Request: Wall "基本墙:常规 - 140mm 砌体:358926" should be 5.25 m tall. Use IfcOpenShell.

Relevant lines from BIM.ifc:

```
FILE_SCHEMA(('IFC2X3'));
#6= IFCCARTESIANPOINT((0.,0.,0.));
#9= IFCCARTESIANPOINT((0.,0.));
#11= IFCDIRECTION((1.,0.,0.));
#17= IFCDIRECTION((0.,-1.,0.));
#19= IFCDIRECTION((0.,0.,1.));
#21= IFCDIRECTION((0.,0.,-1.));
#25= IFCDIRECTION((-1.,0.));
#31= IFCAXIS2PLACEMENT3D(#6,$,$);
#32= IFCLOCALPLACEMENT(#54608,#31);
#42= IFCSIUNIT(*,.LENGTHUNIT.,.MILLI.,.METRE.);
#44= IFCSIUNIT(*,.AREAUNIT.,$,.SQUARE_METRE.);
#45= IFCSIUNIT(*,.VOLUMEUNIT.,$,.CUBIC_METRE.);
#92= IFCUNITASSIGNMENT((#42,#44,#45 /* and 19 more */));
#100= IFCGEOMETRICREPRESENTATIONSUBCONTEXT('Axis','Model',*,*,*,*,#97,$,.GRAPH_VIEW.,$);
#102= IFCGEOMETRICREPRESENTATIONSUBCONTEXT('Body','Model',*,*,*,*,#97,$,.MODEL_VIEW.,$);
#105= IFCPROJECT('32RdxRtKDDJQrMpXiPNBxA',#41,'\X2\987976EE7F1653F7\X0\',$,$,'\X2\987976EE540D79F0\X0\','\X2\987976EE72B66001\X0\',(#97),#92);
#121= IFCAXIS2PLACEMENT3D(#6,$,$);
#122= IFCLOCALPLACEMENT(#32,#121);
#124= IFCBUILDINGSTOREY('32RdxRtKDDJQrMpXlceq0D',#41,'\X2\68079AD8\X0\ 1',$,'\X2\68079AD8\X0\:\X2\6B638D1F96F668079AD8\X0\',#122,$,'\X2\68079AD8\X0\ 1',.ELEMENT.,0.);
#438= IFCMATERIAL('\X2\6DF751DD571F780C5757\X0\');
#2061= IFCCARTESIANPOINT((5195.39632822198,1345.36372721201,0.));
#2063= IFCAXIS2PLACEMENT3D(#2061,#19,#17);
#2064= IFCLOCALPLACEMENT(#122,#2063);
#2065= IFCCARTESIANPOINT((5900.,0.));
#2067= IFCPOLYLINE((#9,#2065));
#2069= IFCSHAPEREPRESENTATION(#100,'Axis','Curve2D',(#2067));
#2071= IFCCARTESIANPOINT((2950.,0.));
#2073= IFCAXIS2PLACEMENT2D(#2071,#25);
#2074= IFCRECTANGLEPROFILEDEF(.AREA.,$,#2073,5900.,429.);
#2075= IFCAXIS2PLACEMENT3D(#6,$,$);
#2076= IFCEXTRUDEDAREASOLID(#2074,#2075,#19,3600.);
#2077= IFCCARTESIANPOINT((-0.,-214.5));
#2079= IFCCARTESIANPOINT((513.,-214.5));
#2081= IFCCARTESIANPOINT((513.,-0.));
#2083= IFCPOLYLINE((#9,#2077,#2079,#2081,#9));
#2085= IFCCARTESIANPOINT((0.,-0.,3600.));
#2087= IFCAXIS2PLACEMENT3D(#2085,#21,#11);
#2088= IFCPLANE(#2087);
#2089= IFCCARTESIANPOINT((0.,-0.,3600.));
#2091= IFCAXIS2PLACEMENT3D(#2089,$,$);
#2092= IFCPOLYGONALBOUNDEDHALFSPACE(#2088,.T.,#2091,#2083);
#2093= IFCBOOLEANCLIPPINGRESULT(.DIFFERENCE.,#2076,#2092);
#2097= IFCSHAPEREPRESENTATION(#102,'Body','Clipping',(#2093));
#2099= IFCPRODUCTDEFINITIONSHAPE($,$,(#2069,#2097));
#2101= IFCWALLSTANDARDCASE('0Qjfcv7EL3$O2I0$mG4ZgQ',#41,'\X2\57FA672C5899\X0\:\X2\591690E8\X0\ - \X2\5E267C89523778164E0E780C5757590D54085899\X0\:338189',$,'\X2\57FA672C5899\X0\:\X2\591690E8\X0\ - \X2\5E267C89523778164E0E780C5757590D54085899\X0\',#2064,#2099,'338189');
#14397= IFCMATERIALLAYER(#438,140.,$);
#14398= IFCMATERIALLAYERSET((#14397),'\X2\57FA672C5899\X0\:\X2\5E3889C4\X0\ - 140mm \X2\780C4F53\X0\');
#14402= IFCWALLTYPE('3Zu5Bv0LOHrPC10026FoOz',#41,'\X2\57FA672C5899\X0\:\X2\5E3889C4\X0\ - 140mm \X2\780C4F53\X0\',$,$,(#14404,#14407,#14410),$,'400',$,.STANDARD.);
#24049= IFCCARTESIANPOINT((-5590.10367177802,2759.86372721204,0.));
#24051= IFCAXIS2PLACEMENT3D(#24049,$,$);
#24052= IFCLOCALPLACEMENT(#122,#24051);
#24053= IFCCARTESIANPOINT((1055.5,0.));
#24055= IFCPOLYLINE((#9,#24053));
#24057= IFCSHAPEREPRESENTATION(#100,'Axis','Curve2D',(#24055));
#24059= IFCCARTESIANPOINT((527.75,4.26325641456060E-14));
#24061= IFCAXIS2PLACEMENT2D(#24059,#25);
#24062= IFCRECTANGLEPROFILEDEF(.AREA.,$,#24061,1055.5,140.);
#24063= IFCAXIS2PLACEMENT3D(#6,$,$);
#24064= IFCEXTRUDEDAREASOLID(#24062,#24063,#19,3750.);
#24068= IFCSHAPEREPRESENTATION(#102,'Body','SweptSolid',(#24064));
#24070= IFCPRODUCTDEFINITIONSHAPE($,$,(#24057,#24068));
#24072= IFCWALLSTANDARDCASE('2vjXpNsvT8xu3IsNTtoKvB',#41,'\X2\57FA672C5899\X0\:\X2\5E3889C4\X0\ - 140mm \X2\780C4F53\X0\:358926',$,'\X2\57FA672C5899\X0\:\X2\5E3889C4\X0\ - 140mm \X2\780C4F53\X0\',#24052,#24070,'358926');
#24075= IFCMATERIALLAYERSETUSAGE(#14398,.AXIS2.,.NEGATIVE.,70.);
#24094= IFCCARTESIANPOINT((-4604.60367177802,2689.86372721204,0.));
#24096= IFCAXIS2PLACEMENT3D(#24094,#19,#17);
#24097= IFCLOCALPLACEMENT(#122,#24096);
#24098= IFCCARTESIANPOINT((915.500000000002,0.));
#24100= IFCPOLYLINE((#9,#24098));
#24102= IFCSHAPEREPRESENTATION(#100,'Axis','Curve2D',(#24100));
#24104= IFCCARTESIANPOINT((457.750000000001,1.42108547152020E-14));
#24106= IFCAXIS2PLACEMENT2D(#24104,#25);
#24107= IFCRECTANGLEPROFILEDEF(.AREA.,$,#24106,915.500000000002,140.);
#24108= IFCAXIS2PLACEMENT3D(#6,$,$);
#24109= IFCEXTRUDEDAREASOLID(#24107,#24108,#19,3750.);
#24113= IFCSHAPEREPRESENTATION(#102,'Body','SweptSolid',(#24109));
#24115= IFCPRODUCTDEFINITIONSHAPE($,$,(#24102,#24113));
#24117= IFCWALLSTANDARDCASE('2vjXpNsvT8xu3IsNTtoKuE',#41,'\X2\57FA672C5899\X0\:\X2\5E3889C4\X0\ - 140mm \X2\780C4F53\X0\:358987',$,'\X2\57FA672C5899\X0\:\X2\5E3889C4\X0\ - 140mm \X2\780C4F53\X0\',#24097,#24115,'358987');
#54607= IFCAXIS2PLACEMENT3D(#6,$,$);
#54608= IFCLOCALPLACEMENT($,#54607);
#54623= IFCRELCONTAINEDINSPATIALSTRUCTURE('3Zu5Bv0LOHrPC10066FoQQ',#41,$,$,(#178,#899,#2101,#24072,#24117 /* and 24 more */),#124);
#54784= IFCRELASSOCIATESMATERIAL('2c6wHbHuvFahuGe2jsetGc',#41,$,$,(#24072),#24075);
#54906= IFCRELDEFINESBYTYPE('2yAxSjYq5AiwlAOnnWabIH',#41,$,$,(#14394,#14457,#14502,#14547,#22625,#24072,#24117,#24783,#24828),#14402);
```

```python
import ifcopenshell
import ifcopenshell.geom
import ifcopenshell.util.representation
import ifcopenshell.util.shape
import ifcopenshell.util.unit

model = ifcopenshell.open("BIM.ifc")
unit_scale = ifcopenshell.util.unit.calculate_unit_scale(model)
settings = ifcopenshell.geom.settings()


def volume(element):
    """Net volume in cubic metres, openings subtracted."""
    shape = ifcopenshell.geom.create_shape(settings, element)
    return ifcopenshell.util.shape.get_volume(shape.geometry)


wall = model.by_guid("2vjXpNsvT8xu3IsNTtoKvB")
before = volume(wall)

body = ifcopenshell.util.representation.get_representation(wall, "Model", "Body")
solid = body.Items[0]
old_height = solid.Depth
solid.Depth = 5.25 / unit_scale
after = volume(wall)

print(f"height {old_height:g} -> {solid.Depth:g}, volume {before:.3f} -> {after:.3f} m3")

model.write("BIM-out.ifc")
```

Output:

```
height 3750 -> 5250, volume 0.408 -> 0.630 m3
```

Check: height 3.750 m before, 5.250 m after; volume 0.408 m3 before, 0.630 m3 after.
